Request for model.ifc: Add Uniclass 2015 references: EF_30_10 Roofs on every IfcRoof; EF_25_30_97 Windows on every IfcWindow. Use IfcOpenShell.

First a look at what the model holds.

```python
import ifcopenshell

model = ifcopenshell.open("model.ifc")
print(model.schema)
print("classifications:", [c.Name for c in model.by_type("IfcClassification")])
for ifc_class in ("IfcDoor", "IfcRoof", "IfcStair", "IfcWall", "IfcWindow"):
    print(ifc_class, len(model.by_type(ifc_class)))
```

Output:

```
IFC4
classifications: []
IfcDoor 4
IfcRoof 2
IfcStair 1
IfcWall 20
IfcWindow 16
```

```python
import ifcopenshell
import ifcopenshell.api.classification

model = ifcopenshell.open("model.ifc")

system = ifcopenshell.api.classification.add_classification(model, classification="Uniclass 2015")

codes = {
    "IfcRoof": ("EF_30_10", "Roofs"),
    "IfcWindow": ("EF_25_30_97", "Windows"),
}
for ifc_class, (code, name) in codes.items():
    products = model.by_type(ifc_class)
    ifcopenshell.api.classification.add_reference(
        model, products=products, classification=system, identification=code, name=name
    )
    print(code, len(products))

model.write("model_v2.ifc")
```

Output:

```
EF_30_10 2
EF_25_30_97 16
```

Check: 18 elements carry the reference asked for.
